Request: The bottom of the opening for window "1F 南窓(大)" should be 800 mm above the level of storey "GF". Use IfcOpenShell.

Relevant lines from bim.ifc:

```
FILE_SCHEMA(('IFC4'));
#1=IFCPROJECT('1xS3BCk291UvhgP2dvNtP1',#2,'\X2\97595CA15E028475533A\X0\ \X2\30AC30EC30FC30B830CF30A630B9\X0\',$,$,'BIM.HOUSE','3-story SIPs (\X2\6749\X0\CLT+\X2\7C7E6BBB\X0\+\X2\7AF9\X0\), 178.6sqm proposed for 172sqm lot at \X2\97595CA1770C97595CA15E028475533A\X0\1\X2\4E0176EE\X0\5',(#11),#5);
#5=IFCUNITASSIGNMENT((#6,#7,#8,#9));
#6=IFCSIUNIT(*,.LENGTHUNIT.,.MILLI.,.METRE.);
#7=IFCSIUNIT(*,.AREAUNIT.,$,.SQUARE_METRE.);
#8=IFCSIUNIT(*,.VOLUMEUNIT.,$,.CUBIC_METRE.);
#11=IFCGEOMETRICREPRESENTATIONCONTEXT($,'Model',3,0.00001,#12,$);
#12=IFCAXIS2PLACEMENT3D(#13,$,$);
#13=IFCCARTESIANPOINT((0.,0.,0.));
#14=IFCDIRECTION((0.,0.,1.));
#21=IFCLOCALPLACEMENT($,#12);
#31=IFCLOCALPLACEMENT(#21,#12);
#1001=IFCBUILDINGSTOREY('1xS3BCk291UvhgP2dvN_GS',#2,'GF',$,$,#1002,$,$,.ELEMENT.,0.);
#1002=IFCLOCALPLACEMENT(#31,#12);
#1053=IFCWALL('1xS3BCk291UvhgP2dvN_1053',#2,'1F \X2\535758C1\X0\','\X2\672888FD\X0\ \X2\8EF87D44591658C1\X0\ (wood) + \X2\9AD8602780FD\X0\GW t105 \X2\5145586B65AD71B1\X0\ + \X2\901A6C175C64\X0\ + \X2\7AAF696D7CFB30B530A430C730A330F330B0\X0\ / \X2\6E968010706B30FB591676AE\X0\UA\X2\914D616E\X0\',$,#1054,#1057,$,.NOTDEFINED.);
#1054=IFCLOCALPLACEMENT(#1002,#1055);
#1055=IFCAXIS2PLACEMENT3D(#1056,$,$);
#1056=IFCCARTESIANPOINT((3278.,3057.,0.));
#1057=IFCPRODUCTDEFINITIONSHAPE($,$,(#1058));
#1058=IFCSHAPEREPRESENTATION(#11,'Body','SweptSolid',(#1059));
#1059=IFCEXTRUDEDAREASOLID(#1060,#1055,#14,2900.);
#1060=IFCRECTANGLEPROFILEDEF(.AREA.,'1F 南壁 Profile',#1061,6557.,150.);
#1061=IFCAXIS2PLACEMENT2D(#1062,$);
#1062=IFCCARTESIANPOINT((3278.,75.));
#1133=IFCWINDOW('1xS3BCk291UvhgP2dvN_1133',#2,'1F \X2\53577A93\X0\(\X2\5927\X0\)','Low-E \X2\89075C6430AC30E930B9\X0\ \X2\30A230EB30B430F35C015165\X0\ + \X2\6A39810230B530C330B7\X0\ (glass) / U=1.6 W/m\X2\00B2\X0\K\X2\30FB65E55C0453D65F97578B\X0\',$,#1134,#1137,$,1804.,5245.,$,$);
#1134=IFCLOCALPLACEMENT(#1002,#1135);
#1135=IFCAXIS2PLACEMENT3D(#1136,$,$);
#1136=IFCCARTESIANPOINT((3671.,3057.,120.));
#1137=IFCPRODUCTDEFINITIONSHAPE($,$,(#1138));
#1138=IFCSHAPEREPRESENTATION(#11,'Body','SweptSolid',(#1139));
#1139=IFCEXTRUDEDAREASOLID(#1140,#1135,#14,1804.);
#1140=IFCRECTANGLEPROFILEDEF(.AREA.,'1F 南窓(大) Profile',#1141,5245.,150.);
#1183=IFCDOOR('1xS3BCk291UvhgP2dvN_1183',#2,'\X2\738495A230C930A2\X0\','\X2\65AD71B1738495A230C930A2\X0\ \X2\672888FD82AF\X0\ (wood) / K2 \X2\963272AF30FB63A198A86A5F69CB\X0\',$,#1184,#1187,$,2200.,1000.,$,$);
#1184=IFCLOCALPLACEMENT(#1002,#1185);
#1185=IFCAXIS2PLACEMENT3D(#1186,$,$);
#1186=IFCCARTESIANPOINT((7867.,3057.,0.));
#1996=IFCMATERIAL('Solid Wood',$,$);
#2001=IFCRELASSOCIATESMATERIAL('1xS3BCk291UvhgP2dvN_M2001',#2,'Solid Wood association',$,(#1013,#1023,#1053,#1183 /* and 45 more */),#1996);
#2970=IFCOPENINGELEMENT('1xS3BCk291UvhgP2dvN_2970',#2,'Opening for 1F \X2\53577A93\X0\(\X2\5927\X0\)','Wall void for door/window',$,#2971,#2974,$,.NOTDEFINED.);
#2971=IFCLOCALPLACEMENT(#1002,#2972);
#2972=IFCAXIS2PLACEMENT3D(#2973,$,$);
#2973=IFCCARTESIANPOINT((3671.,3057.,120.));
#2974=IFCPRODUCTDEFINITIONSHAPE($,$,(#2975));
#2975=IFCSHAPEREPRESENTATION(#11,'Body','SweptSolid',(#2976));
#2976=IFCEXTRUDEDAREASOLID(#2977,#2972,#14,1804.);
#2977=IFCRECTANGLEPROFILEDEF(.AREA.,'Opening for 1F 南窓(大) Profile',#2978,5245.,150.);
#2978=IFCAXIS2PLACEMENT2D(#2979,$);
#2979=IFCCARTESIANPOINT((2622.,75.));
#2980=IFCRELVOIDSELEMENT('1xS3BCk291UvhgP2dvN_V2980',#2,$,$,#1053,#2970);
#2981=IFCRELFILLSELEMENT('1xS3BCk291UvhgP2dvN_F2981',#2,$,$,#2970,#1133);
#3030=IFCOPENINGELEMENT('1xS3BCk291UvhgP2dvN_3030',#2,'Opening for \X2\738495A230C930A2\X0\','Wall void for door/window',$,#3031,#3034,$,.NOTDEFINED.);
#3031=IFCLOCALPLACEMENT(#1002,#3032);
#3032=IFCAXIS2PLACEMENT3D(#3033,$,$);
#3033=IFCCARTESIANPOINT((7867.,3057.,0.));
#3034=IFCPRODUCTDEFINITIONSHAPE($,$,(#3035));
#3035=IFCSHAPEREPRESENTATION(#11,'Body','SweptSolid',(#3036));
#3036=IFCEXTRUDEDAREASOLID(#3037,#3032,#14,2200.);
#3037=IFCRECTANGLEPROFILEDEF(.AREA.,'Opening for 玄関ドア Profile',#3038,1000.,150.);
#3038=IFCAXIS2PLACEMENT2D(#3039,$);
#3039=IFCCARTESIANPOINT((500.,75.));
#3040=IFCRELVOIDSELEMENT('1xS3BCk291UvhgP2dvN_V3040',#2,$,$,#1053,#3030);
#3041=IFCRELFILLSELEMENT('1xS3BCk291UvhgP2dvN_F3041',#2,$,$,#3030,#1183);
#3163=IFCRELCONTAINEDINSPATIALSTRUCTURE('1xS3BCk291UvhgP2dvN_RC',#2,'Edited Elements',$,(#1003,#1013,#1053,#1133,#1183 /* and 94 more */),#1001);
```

```python
import numpy as np
import ifcopenshell
import ifcopenshell.api.geometry
import ifcopenshell.geom
import ifcopenshell.util.element
import ifcopenshell.util.placement
import ifcopenshell.util.shape
import ifcopenshell.util.unit

model = ifcopenshell.open("bim.ifc")
unit_scale = ifcopenshell.util.unit.calculate_unit_scale(model)

window = model.by_id(1133)
opening = window.FillsVoids[0].RelatingOpeningElement
storey = ifcopenshell.util.element.get_container(window, ifc_class="IfcBuildingStorey")
level = ifcopenshell.util.placement.get_local_placement(storey.ObjectPlacement)[2, 3]

# The opening's origin need not be at the sill, so measure its lowest point.
shape = ifcopenshell.geom.create_shape(ifcopenshell.geom.settings(), opening)
bottom = ifcopenshell.util.shape.get_shape_bottom_elevation(shape, shape.geometry) / unit_scale
dz = level + 800.0 - bottom

shift = np.array([0.0, 0.0, dz])
# The window is not placed relative to its opening, so move both.
for product in (opening, window):
    matrix = ifcopenshell.util.placement.get_local_placement(product.ObjectPlacement)
    matrix[:3, 3] += shift
    ifcopenshell.api.geometry.edit_object_placement(model, product=product, matrix=matrix, is_si=False)

print(f"moved by {dz * unit_scale:+.3f} m")

model.write("bim_rev.ifc")
```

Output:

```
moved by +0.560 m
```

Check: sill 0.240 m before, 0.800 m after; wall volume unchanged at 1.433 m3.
